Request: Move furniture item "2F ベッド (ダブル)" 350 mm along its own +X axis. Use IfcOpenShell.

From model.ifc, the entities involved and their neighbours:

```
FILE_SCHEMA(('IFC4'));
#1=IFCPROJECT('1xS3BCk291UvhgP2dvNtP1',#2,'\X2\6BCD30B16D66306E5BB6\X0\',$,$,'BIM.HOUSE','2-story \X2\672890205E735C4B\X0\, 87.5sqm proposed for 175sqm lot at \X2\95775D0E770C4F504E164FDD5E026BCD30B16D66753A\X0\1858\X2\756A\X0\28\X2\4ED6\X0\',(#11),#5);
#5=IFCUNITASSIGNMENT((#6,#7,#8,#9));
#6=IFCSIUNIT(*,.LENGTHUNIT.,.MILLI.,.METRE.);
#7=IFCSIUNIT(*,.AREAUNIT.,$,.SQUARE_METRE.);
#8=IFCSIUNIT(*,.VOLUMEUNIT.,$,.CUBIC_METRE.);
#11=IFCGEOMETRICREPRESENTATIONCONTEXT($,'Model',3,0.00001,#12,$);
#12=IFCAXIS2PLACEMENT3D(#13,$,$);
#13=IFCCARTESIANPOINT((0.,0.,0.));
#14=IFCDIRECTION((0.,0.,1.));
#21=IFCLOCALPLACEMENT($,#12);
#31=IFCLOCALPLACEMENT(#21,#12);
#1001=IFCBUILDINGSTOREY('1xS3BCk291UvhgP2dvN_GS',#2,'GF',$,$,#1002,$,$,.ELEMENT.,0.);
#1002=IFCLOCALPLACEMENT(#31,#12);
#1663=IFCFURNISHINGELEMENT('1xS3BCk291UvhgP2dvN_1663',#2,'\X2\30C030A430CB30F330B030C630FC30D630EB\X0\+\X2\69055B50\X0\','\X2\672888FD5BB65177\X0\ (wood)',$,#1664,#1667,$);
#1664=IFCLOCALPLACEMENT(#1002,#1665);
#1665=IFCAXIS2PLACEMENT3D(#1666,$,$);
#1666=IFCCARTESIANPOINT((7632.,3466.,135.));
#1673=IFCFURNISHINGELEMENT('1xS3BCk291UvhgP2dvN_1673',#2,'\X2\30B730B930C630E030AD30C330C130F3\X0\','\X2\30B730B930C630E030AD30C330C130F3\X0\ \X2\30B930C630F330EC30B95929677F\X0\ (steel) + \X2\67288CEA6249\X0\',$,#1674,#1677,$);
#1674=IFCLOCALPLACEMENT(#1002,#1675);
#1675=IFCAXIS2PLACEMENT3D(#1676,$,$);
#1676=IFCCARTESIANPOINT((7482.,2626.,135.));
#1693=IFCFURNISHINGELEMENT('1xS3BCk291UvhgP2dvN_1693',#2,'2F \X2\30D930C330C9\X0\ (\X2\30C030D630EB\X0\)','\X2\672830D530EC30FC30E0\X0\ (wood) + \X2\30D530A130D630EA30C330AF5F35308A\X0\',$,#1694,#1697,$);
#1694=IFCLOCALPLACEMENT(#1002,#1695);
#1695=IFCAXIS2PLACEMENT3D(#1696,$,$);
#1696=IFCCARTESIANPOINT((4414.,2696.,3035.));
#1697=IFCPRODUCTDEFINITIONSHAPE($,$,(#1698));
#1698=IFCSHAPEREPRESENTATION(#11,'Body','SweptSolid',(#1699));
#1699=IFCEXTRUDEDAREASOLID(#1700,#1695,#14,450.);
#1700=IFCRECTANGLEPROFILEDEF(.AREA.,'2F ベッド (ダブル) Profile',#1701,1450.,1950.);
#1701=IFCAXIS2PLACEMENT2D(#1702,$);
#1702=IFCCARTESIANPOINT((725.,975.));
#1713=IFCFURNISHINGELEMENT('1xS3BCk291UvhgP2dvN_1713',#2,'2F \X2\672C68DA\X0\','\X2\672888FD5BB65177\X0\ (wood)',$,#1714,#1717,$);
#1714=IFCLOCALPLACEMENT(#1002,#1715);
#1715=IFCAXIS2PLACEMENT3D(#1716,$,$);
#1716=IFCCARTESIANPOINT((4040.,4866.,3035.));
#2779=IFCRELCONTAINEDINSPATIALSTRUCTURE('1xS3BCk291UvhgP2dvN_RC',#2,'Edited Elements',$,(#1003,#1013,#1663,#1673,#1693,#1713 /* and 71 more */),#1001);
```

```python
import ifcopenshell
import ifcopenshell.api.geometry
import ifcopenshell.util.placement

model = ifcopenshell.open("model.ifc")

item = model.by_guid("1xS3BCk291UvhgP2dvN_1693")
matrix = ifcopenshell.util.placement.get_local_placement(item.ObjectPlacement)
matrix[:3, 3] += matrix[:3, 0] * 350.0
ifcopenshell.api.geometry.edit_object_placement(model, product=item, matrix=matrix, is_si=False)

print(ifcopenshell.util.placement.get_local_placement(item.ObjectPlacement).round(3) + 0.0)

model.write("model-out.ifc")
```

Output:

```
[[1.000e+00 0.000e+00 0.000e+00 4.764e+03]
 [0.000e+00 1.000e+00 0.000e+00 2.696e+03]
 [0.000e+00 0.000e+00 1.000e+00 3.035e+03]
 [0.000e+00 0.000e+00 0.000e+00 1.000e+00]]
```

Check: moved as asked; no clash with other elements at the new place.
